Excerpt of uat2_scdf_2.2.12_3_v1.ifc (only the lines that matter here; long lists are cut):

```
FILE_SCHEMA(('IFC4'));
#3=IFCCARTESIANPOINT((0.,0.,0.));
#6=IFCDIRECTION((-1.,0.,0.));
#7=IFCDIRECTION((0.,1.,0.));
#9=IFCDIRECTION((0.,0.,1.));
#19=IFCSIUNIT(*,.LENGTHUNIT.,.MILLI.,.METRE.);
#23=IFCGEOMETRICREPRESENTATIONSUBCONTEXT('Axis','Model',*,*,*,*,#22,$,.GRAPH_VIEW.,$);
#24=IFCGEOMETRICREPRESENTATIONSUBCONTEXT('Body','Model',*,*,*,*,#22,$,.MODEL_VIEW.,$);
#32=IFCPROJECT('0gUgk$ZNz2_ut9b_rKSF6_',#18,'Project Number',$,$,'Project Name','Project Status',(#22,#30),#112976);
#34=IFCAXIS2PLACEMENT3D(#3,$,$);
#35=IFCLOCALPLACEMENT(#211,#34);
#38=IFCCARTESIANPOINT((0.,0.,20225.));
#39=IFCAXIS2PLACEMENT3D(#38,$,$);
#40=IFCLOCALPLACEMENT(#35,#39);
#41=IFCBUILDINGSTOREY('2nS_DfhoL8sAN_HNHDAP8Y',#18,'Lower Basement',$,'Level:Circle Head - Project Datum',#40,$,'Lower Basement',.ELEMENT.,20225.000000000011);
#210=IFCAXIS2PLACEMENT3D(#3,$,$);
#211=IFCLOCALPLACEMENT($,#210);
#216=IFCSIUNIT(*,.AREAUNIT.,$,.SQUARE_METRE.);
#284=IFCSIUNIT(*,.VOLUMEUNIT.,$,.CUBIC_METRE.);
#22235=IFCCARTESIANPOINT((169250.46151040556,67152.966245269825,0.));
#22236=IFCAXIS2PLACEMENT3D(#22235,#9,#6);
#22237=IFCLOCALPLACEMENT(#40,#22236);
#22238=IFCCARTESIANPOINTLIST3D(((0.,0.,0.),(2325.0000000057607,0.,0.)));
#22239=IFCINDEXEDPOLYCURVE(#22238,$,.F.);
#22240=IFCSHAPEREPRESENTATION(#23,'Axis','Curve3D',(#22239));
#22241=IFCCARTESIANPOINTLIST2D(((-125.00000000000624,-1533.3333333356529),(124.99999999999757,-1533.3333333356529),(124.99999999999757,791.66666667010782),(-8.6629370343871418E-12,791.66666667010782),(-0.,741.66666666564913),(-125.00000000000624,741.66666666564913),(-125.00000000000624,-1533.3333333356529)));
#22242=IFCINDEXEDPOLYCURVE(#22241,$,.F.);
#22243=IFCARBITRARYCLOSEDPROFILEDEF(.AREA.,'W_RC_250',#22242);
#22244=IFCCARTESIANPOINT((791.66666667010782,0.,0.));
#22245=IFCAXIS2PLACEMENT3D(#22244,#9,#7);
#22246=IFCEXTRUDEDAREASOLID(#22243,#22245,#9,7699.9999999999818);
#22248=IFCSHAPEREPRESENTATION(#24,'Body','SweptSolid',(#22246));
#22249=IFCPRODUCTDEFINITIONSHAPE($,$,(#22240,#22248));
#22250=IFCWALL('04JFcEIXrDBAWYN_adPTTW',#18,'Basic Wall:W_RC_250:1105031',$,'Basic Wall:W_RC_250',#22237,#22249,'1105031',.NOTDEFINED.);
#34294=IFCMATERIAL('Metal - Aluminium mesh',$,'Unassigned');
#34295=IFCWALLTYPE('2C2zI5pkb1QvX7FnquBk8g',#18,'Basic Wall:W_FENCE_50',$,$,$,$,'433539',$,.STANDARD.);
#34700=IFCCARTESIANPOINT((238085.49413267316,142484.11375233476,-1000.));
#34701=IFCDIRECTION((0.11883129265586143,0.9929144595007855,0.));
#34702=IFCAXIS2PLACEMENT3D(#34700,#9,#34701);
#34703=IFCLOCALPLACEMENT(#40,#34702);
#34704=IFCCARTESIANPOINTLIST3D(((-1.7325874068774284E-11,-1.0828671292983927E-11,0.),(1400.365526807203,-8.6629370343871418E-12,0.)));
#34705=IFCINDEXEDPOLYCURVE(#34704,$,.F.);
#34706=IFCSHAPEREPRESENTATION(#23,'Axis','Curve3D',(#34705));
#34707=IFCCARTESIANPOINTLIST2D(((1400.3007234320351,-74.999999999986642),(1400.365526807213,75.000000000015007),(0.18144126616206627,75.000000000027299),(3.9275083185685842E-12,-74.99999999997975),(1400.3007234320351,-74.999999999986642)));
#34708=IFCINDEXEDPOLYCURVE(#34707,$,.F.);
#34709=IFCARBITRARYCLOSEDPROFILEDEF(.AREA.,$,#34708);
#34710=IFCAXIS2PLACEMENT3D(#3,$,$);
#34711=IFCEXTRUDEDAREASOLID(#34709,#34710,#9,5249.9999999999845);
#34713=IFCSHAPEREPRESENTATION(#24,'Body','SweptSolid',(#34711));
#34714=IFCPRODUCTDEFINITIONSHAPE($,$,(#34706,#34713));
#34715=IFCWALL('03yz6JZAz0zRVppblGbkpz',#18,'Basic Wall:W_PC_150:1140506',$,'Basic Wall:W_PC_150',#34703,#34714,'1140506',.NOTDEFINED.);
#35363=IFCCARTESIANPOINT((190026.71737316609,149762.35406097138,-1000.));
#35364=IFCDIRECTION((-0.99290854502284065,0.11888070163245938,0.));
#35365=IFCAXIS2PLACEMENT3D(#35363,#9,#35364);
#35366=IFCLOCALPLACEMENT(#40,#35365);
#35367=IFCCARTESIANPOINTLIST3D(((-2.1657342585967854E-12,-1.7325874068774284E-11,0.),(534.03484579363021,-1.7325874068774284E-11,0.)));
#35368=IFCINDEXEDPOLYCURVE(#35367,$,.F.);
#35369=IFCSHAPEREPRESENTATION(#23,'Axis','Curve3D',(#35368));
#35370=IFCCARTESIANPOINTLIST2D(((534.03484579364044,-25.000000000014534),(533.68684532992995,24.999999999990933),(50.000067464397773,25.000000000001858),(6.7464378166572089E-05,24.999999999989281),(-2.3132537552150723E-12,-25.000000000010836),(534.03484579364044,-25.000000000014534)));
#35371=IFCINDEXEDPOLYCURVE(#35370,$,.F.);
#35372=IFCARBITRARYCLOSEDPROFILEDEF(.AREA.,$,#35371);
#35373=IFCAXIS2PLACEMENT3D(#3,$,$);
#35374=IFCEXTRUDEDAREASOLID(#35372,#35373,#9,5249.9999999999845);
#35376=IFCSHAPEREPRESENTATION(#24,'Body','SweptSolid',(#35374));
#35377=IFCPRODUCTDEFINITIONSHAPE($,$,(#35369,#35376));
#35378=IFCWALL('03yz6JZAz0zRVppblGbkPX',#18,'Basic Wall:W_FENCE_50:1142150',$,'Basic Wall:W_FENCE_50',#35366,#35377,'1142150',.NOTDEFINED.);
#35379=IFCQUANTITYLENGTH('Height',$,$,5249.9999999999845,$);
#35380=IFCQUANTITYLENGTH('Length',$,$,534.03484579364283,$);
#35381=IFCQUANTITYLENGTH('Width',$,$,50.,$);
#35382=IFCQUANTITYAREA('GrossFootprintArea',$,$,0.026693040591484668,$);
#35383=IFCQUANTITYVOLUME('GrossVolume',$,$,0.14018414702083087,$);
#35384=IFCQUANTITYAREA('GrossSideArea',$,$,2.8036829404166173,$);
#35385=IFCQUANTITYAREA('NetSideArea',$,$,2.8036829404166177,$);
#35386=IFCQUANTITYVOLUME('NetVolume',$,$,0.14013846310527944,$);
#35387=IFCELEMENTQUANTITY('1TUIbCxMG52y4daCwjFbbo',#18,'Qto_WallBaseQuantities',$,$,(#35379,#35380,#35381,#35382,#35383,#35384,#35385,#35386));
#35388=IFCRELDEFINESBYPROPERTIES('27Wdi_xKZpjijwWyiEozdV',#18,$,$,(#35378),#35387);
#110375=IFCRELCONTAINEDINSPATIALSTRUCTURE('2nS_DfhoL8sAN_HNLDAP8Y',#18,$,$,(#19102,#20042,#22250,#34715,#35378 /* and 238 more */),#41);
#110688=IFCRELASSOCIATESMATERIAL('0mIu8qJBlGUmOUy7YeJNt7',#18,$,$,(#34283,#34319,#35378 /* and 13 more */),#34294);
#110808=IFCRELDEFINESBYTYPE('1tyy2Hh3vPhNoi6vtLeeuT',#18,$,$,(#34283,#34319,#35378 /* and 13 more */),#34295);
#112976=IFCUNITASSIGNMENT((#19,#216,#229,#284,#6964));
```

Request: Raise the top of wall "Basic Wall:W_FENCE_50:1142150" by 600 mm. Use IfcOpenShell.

```python
import ifcopenshell
import ifcopenshell.api.pset
import ifcopenshell.geom
import ifcopenshell.util.element
import ifcopenshell.util.representation
import ifcopenshell.util.shape
import ifcopenshell.util.unit

model = ifcopenshell.open("uat2_scdf_2.2.12_3_v1.ifc")
unit_scale = ifcopenshell.util.unit.calculate_unit_scale(model)
area_scale = ifcopenshell.util.unit.calculate_unit_scale(model, "AREAUNIT")
volume_scale = ifcopenshell.util.unit.calculate_unit_scale(model, "VOLUMEUNIT")
settings = ifcopenshell.geom.settings()


def volume(element):
    """Net volume in cubic metres, openings subtracted."""
    shape = ifcopenshell.geom.create_shape(settings, element)
    return ifcopenshell.util.shape.get_volume(shape.geometry)


wall = model.by_guid("03yz6JZAz0zRVppblGbkPX")
before = volume(wall)

body = ifcopenshell.util.representation.get_representation(wall, "Model", "Body")
solid = body.Items[0]
old_height = solid.Depth
solid.Depth += 600.0
after = volume(wall)
thickness = 0.05  # wall thickness in metres

# Update the stored height, areas and volumes.
qto = model.by_id(ifcopenshell.util.element.get_pset(wall, "Qto_WallBaseQuantities", should_inherit=False)["id"])
ifcopenshell.api.pset.edit_qto(model, qto=qto, properties={
    "Height": solid.Depth,
    "GrossVolume": ifcopenshell.util.element.get_pset(wall, "Qto_WallBaseQuantities", "GrossVolume") * solid.Depth / old_height,
    "GrossSideArea": ifcopenshell.util.element.get_pset(wall, "Qto_WallBaseQuantities", "GrossSideArea") * solid.Depth / old_height,
    "NetSideArea": after / thickness / area_scale,
    "NetVolume": after / volume_scale,
})

print(f"height {old_height:g} -> {solid.Depth:g}, volume {before:.3f} -> {after:.3f} m3")

model.write("uat2_scdf_2.2.12_3_v1_edited.ifc")
```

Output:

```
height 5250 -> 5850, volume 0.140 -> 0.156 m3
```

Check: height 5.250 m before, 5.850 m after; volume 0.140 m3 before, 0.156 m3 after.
